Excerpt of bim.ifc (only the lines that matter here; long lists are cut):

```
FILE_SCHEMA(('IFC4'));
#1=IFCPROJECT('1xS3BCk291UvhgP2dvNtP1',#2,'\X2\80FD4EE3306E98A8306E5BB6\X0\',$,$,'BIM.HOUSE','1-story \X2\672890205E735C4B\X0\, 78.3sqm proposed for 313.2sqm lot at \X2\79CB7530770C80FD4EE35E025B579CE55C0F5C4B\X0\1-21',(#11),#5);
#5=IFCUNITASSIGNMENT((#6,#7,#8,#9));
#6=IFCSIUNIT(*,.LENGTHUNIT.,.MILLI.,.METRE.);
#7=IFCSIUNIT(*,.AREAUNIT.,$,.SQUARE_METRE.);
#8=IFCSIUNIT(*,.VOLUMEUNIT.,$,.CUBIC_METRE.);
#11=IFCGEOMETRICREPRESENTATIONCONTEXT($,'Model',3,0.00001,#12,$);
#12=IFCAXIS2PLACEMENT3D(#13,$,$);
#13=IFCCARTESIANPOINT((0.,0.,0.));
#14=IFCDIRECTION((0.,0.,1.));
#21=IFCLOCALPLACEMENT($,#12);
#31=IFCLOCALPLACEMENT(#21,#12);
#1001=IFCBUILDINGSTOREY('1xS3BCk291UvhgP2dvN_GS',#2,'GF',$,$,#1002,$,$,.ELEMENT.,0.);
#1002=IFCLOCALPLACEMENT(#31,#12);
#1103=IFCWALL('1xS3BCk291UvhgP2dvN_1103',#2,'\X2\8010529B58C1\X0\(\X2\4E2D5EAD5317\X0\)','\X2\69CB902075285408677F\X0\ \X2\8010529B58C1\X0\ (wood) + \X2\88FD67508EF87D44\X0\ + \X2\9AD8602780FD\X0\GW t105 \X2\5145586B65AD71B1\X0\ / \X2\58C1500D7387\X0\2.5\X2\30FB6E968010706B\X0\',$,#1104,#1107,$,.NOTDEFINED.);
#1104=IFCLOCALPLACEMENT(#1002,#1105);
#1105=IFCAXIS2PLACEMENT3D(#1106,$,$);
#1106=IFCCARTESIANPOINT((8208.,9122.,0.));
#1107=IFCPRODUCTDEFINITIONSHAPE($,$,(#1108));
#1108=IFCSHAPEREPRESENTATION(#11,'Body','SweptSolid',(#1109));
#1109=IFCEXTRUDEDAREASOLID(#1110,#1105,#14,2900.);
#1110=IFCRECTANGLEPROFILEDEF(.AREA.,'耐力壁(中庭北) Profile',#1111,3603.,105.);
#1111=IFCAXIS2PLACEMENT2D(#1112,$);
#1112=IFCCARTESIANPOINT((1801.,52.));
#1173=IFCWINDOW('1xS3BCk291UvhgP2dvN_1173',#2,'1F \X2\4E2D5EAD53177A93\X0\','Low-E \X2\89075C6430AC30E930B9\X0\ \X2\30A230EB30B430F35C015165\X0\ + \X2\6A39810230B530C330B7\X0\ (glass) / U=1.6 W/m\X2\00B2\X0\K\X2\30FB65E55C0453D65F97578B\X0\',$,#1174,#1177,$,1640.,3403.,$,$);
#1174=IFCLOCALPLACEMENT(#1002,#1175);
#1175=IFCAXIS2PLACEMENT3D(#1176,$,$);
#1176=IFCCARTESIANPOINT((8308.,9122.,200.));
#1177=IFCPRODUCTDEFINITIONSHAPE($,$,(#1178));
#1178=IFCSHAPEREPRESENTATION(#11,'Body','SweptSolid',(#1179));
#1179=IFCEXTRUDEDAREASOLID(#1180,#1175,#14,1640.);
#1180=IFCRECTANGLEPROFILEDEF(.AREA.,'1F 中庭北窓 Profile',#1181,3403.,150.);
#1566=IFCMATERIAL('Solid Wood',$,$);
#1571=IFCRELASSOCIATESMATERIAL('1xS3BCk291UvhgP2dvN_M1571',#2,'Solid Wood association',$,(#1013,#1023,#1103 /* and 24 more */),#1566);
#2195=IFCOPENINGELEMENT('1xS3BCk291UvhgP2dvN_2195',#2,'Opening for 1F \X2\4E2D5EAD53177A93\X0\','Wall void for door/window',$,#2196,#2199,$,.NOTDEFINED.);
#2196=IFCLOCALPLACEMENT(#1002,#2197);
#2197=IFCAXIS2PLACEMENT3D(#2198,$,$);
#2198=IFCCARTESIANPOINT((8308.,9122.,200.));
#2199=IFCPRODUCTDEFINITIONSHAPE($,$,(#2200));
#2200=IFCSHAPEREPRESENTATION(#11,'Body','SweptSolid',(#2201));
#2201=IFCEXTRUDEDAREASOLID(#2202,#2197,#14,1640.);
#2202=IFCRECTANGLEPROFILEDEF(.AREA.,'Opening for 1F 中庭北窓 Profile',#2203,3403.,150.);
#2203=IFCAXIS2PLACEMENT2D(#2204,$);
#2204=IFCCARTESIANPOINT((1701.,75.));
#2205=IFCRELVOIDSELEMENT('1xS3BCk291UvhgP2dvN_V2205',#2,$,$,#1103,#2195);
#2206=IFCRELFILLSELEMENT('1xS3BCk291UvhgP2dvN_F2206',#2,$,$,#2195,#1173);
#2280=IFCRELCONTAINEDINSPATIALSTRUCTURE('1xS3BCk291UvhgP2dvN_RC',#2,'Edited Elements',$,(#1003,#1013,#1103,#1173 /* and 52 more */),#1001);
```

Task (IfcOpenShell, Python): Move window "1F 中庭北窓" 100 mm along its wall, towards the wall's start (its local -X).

```python
import ifcopenshell
import ifcopenshell.api.geometry
import ifcopenshell.util.placement

model = ifcopenshell.open("bim.ifc")

window = model.by_id(1173)
opening = window.FillsVoids[0].RelatingOpeningElement
wall = opening.VoidsElements[0].RelatingBuildingElement

wall_matrix = ifcopenshell.util.placement.get_local_placement(wall.ObjectPlacement)
shift = wall_matrix[:3, 0] * -100.0
before = ifcopenshell.util.placement.get_local_placement(window.ObjectPlacement)[:3, 3].copy()

# The window is not placed relative to its opening, so move both.
for product in (opening, window):
    matrix = ifcopenshell.util.placement.get_local_placement(product.ObjectPlacement)
    matrix[:3, 3] += shift
    ifcopenshell.api.geometry.edit_object_placement(model, product=product, matrix=matrix, is_si=False)

after = ifcopenshell.util.placement.get_local_placement(window.ObjectPlacement)[:3, 3]
print("window moved by", (after - before).round(3) + 0.0)

model.write("bim_edited.ifc")
```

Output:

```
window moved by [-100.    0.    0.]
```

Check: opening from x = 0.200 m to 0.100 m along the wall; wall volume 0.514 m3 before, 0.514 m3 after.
